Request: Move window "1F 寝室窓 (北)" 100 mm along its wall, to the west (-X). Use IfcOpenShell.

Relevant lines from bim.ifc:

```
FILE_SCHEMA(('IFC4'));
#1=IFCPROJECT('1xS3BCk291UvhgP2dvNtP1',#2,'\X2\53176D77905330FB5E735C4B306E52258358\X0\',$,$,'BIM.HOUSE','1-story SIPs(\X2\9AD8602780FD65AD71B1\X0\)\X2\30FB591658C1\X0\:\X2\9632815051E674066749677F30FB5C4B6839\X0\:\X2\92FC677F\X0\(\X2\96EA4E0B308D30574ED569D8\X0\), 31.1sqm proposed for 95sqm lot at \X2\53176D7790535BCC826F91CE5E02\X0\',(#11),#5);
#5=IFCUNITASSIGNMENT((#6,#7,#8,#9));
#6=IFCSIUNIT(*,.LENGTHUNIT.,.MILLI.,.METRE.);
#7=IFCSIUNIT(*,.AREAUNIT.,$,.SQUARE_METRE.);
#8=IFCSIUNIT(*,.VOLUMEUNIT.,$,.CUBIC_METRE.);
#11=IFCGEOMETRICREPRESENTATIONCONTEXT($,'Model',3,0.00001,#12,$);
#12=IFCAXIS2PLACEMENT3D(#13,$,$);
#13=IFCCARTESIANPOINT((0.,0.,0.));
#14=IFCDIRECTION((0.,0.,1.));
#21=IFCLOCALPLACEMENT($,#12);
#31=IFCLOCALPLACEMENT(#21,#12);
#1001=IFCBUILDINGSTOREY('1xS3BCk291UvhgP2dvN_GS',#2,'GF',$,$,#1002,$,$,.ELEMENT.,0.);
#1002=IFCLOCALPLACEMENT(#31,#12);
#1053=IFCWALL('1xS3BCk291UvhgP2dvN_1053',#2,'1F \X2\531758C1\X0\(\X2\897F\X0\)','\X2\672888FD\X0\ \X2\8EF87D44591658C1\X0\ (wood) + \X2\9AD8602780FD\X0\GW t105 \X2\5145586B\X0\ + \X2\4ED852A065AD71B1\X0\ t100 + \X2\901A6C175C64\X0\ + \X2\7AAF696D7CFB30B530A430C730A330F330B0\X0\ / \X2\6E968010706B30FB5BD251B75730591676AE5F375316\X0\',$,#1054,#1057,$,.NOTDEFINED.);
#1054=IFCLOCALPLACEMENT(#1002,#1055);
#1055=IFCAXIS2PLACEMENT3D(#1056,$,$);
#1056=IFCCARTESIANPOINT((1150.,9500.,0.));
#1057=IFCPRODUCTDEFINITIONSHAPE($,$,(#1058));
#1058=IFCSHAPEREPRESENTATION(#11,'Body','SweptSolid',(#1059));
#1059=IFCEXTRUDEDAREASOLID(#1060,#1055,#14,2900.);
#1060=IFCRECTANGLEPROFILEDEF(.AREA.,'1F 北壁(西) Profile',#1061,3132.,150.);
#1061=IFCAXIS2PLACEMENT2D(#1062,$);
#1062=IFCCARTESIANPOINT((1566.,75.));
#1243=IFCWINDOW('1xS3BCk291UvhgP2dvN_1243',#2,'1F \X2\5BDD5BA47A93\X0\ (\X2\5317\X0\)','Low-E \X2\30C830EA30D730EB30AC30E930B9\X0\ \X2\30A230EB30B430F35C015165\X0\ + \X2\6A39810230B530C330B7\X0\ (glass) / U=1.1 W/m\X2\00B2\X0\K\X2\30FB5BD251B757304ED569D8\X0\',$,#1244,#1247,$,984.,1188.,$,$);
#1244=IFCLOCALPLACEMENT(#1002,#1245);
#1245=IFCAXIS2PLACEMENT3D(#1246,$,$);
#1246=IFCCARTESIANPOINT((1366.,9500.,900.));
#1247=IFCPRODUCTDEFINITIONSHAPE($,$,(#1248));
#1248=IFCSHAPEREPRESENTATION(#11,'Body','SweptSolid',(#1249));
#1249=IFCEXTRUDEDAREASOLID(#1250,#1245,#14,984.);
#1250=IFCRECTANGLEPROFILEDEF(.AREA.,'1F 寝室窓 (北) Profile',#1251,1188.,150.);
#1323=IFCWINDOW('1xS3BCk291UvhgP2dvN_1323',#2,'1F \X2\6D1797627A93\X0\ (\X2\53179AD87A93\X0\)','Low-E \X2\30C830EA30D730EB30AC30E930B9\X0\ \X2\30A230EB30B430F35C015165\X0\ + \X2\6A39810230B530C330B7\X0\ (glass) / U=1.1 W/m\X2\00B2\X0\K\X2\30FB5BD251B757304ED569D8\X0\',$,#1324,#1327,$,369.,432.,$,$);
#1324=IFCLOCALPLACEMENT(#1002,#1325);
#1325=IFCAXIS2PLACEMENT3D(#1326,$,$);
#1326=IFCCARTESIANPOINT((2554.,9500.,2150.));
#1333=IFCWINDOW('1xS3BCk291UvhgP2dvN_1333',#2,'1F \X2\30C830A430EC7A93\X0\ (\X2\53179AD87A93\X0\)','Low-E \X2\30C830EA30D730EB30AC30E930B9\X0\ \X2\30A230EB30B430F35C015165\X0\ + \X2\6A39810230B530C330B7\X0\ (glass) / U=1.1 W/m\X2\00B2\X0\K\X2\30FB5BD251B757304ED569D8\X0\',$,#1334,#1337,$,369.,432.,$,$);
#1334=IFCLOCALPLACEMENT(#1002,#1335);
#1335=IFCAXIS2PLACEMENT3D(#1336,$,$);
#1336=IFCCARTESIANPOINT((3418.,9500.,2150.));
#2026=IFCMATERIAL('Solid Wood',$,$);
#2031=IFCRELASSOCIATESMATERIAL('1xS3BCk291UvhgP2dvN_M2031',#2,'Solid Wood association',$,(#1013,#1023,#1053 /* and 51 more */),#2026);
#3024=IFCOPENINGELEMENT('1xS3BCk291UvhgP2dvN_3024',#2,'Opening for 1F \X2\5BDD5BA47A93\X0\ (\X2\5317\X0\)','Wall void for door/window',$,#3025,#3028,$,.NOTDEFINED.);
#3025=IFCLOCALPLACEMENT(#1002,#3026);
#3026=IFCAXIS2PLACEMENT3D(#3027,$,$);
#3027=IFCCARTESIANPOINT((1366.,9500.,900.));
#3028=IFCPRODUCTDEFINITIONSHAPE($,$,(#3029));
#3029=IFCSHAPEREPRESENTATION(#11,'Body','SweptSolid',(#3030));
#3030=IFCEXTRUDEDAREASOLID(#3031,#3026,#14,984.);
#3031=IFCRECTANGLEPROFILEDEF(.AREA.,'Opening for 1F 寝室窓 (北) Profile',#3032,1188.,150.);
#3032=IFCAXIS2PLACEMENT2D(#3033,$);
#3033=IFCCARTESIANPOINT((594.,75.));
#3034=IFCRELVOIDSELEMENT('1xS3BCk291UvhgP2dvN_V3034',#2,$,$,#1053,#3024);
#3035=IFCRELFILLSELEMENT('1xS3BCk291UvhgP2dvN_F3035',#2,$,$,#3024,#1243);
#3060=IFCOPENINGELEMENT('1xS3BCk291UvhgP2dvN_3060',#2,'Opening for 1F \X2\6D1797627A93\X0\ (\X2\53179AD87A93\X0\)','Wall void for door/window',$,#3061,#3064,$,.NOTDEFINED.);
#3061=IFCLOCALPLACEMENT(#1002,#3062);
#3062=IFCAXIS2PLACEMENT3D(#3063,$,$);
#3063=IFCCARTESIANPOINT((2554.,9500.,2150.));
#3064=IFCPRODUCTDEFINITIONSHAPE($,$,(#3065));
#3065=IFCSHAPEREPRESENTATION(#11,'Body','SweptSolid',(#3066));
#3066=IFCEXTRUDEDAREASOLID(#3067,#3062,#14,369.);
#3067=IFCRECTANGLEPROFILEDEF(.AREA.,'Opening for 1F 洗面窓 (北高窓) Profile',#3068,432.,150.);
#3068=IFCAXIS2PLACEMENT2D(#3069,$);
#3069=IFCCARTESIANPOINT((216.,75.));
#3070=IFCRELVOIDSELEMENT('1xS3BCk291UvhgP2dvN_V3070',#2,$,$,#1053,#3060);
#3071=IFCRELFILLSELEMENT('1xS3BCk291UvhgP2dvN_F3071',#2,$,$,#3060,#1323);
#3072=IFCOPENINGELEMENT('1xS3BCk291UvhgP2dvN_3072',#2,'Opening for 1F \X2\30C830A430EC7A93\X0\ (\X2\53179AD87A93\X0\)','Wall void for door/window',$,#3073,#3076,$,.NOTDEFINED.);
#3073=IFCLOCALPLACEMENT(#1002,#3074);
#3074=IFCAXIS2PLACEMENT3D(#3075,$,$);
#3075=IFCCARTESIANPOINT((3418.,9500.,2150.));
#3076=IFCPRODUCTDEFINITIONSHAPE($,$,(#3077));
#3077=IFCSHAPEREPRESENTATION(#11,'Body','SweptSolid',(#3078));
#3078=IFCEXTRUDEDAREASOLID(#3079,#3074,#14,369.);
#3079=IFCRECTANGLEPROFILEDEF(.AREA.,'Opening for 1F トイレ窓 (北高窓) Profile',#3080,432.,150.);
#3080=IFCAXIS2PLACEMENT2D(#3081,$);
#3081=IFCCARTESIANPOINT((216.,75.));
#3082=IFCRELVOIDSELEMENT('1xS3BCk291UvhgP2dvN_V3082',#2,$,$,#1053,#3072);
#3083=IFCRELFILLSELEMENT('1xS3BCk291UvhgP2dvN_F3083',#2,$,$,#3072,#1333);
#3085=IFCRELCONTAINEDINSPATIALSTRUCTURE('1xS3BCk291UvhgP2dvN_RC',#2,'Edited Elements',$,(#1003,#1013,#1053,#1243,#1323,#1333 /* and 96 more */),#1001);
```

```python
import ifcopenshell
import ifcopenshell.api.geometry
import ifcopenshell.util.placement
import ifcopenshell.util.unit

model = ifcopenshell.open("bim.ifc")
unit_scale = ifcopenshell.util.unit.calculate_unit_scale(model)

window = model.by_guid("1xS3BCk291UvhgP2dvN_1243")
opening = window.FillsVoids[0].RelatingOpeningElement
wall = opening.VoidsElements[0].RelatingBuildingElement

wall_matrix = ifcopenshell.util.placement.get_local_placement(wall.ObjectPlacement)
shift = wall_matrix[:3, 0] * -0.1 / unit_scale
before = ifcopenshell.util.placement.get_local_placement(window.ObjectPlacement)[:3, 3].copy()

# The window is not placed relative to its opening, so move both.
for product in (opening, window):
    matrix = ifcopenshell.util.placement.get_local_placement(product.ObjectPlacement)
    matrix[:3, 3] += shift
    ifcopenshell.api.geometry.edit_object_placement(model, product=product, matrix=matrix, is_si=False)

after = ifcopenshell.util.placement.get_local_placement(window.ObjectPlacement)[:3, 3]
print("window moved by", (after - before).round(3) + 0.0)

model.write("bim_edited.ifc")
```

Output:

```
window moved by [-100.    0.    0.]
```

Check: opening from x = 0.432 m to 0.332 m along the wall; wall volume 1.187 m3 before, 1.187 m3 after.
